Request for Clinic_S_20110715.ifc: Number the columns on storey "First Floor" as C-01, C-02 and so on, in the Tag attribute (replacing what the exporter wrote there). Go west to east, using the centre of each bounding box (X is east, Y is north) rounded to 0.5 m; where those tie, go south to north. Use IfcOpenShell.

First a look at what the model holds.

```python
import ifcopenshell
import ifcopenshell.util.element
import ifcopenshell.util.placement

model = ifcopenshell.open("Clinic_S_20110715.ifc")
print(model.schema)
storey = next(s for s in model.by_type("IfcBuildingStorey") if s.Name == "First Floor")
columns = [e for e in ifcopenshell.util.element.get_decomposition(storey) if e.is_a("IfcColumn")]
for e in sorted(columns, key=lambda e: e.id()):
    origin = ifcopenshell.util.placement.get_local_placement(e.ObjectPlacement)[:3, 3]
    print(e.id(), e.Tag, e.Name, origin.round(2) + 0.0, sep=" | ")
```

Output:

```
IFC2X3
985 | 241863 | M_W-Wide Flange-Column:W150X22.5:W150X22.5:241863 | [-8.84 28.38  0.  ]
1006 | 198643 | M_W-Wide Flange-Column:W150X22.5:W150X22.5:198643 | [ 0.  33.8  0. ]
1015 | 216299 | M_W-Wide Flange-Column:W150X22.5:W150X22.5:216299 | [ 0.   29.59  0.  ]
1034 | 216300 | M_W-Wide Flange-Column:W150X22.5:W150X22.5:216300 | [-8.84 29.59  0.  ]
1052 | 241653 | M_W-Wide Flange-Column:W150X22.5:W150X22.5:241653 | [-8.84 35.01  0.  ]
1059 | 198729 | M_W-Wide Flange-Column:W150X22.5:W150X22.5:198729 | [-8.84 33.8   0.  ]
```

```python
import ifcopenshell
import ifcopenshell.geom
import ifcopenshell.util.element
import ifcopenshell.util.shape

model = ifcopenshell.open("Clinic_S_20110715.ifc")
settings = ifcopenshell.geom.settings()
settings.set("use-world-coords", True)


def centre(element):
    shape = ifcopenshell.geom.create_shape(settings, element)
    return ifcopenshell.util.shape.get_bbox_centroid(shape.geometry)


storey = next(s for s in model.by_type("IfcBuildingStorey") if s.Name == "First Floor")
columns = [e for e in ifcopenshell.util.element.get_decomposition(storey) if e.is_a("IfcColumn")]

# Insertion points can sit at a corner or the storey origin, so sort by the geometry (in metres).
centres = {e: centre(e) for e in columns}
columns.sort(key=lambda e: (round(centres[e][0] / 0.5), centres[e][1]))

for i, e in enumerate(columns, start=1):
    number = f"C-{i:02d}"
    e.Tag = number
    print(e.id(), number)

model.write("Clinic_S_20110715-out.ifc")
```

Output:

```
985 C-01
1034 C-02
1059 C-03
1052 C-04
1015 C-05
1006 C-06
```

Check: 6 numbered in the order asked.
